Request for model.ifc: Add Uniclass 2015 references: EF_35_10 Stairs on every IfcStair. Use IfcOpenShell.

First a look at what the model holds.

```python
import ifcopenshell

model = ifcopenshell.open("model.ifc")
print(model.schema)
print("classifications:", [c.Name for c in model.by_type("IfcClassification")])
for ifc_class in ("IfcDoor", "IfcRoof", "IfcStair", "IfcWall", "IfcWindow"):
    print(ifc_class, len(model.by_type(ifc_class)))
```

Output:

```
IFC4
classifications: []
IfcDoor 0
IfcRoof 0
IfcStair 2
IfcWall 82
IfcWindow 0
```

```python
import ifcopenshell
import ifcopenshell.api.classification

model = ifcopenshell.open("model.ifc")

system = ifcopenshell.api.classification.add_classification(model, classification="Uniclass 2015")

codes = {
    "IfcStair": ("EF_35_10", "Stairs"),
}
for ifc_class, (code, name) in codes.items():
    products = model.by_type(ifc_class)
    ifcopenshell.api.classification.add_reference(
        model, products=products, classification=system, identification=code, name=name
    )
    print(code, len(products))

model.write("model-out.ifc")
```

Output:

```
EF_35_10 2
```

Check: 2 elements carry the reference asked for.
